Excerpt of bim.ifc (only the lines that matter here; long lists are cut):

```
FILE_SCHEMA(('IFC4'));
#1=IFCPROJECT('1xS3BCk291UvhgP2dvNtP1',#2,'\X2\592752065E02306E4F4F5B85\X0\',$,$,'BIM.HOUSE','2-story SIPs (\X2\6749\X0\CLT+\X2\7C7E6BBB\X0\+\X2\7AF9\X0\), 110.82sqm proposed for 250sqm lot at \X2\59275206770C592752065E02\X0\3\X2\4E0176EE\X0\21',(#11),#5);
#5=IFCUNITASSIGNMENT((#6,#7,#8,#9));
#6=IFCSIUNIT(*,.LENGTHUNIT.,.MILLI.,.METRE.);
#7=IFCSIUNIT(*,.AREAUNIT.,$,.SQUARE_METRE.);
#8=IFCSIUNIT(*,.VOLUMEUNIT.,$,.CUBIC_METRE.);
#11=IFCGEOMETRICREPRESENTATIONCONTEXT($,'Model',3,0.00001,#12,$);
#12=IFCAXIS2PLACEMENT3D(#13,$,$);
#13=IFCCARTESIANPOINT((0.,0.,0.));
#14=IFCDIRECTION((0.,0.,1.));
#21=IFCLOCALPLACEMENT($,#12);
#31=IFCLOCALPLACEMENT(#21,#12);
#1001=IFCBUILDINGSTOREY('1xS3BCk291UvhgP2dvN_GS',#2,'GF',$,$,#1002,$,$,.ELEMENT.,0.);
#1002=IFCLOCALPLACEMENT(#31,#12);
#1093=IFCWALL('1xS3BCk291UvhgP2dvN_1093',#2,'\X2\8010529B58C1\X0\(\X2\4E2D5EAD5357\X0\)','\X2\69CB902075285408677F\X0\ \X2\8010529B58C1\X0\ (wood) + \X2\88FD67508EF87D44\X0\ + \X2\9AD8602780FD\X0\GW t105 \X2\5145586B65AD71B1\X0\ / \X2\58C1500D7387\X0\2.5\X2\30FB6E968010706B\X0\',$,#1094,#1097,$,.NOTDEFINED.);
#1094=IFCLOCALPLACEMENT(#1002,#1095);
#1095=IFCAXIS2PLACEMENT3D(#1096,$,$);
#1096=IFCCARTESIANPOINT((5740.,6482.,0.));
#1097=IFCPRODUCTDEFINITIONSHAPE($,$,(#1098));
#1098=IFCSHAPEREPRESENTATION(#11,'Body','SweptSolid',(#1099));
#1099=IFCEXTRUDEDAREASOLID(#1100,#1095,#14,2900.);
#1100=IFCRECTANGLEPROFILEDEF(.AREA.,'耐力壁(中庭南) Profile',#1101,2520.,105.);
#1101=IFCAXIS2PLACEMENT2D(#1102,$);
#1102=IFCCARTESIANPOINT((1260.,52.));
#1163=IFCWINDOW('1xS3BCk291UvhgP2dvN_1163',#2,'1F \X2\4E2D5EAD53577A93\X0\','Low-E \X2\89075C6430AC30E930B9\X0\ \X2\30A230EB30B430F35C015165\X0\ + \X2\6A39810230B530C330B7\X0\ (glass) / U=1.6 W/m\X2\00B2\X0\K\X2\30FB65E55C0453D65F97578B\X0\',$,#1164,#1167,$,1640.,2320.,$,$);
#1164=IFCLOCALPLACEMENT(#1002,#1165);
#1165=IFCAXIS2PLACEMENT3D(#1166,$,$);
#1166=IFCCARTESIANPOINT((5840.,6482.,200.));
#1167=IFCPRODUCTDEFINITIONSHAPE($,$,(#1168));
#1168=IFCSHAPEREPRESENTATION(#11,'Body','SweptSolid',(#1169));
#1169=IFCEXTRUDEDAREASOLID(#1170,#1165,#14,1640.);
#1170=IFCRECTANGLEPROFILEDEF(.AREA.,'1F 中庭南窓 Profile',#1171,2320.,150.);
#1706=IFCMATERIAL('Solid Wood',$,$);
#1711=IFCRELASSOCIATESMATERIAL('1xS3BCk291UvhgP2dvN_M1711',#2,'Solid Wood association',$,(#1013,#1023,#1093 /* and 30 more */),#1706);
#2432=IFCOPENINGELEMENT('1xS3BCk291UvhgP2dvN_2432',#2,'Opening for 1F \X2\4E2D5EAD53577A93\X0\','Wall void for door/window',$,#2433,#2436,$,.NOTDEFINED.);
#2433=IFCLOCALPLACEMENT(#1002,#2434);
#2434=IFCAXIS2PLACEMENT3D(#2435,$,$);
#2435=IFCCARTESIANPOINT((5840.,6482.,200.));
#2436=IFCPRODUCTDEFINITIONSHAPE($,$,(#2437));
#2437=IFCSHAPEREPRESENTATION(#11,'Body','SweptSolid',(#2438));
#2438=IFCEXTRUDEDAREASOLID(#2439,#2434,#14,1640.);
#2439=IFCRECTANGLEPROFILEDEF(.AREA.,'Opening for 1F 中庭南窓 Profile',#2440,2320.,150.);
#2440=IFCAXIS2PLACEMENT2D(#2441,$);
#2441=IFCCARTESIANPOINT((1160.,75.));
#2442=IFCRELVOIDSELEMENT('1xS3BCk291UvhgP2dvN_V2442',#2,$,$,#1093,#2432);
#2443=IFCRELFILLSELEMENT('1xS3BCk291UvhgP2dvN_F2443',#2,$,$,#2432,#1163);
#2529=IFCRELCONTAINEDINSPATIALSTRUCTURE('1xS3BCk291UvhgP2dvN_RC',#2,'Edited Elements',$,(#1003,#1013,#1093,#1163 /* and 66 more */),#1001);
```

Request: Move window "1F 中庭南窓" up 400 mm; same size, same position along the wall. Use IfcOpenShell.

```python
import numpy as np
import ifcopenshell
import ifcopenshell.api.geometry
import ifcopenshell.util.placement
import ifcopenshell.util.unit

model = ifcopenshell.open("bim.ifc")
unit_scale = ifcopenshell.util.unit.calculate_unit_scale(model)

window = model.by_id(1163)
opening = window.FillsVoids[0].RelatingOpeningElement
dz = 0.4 / unit_scale

shift = np.array([0.0, 0.0, dz])
# The window is not placed relative to its opening, so move both.
for product in (opening, window):
    matrix = ifcopenshell.util.placement.get_local_placement(product.ObjectPlacement)
    matrix[:3, 3] += shift
    ifcopenshell.api.geometry.edit_object_placement(model, product=product, matrix=matrix, is_si=False)

print(f"moved by {dz * unit_scale:+.3f} m")

model.write("bim_edited.ifc")
```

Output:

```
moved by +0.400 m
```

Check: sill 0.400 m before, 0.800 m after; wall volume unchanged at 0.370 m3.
